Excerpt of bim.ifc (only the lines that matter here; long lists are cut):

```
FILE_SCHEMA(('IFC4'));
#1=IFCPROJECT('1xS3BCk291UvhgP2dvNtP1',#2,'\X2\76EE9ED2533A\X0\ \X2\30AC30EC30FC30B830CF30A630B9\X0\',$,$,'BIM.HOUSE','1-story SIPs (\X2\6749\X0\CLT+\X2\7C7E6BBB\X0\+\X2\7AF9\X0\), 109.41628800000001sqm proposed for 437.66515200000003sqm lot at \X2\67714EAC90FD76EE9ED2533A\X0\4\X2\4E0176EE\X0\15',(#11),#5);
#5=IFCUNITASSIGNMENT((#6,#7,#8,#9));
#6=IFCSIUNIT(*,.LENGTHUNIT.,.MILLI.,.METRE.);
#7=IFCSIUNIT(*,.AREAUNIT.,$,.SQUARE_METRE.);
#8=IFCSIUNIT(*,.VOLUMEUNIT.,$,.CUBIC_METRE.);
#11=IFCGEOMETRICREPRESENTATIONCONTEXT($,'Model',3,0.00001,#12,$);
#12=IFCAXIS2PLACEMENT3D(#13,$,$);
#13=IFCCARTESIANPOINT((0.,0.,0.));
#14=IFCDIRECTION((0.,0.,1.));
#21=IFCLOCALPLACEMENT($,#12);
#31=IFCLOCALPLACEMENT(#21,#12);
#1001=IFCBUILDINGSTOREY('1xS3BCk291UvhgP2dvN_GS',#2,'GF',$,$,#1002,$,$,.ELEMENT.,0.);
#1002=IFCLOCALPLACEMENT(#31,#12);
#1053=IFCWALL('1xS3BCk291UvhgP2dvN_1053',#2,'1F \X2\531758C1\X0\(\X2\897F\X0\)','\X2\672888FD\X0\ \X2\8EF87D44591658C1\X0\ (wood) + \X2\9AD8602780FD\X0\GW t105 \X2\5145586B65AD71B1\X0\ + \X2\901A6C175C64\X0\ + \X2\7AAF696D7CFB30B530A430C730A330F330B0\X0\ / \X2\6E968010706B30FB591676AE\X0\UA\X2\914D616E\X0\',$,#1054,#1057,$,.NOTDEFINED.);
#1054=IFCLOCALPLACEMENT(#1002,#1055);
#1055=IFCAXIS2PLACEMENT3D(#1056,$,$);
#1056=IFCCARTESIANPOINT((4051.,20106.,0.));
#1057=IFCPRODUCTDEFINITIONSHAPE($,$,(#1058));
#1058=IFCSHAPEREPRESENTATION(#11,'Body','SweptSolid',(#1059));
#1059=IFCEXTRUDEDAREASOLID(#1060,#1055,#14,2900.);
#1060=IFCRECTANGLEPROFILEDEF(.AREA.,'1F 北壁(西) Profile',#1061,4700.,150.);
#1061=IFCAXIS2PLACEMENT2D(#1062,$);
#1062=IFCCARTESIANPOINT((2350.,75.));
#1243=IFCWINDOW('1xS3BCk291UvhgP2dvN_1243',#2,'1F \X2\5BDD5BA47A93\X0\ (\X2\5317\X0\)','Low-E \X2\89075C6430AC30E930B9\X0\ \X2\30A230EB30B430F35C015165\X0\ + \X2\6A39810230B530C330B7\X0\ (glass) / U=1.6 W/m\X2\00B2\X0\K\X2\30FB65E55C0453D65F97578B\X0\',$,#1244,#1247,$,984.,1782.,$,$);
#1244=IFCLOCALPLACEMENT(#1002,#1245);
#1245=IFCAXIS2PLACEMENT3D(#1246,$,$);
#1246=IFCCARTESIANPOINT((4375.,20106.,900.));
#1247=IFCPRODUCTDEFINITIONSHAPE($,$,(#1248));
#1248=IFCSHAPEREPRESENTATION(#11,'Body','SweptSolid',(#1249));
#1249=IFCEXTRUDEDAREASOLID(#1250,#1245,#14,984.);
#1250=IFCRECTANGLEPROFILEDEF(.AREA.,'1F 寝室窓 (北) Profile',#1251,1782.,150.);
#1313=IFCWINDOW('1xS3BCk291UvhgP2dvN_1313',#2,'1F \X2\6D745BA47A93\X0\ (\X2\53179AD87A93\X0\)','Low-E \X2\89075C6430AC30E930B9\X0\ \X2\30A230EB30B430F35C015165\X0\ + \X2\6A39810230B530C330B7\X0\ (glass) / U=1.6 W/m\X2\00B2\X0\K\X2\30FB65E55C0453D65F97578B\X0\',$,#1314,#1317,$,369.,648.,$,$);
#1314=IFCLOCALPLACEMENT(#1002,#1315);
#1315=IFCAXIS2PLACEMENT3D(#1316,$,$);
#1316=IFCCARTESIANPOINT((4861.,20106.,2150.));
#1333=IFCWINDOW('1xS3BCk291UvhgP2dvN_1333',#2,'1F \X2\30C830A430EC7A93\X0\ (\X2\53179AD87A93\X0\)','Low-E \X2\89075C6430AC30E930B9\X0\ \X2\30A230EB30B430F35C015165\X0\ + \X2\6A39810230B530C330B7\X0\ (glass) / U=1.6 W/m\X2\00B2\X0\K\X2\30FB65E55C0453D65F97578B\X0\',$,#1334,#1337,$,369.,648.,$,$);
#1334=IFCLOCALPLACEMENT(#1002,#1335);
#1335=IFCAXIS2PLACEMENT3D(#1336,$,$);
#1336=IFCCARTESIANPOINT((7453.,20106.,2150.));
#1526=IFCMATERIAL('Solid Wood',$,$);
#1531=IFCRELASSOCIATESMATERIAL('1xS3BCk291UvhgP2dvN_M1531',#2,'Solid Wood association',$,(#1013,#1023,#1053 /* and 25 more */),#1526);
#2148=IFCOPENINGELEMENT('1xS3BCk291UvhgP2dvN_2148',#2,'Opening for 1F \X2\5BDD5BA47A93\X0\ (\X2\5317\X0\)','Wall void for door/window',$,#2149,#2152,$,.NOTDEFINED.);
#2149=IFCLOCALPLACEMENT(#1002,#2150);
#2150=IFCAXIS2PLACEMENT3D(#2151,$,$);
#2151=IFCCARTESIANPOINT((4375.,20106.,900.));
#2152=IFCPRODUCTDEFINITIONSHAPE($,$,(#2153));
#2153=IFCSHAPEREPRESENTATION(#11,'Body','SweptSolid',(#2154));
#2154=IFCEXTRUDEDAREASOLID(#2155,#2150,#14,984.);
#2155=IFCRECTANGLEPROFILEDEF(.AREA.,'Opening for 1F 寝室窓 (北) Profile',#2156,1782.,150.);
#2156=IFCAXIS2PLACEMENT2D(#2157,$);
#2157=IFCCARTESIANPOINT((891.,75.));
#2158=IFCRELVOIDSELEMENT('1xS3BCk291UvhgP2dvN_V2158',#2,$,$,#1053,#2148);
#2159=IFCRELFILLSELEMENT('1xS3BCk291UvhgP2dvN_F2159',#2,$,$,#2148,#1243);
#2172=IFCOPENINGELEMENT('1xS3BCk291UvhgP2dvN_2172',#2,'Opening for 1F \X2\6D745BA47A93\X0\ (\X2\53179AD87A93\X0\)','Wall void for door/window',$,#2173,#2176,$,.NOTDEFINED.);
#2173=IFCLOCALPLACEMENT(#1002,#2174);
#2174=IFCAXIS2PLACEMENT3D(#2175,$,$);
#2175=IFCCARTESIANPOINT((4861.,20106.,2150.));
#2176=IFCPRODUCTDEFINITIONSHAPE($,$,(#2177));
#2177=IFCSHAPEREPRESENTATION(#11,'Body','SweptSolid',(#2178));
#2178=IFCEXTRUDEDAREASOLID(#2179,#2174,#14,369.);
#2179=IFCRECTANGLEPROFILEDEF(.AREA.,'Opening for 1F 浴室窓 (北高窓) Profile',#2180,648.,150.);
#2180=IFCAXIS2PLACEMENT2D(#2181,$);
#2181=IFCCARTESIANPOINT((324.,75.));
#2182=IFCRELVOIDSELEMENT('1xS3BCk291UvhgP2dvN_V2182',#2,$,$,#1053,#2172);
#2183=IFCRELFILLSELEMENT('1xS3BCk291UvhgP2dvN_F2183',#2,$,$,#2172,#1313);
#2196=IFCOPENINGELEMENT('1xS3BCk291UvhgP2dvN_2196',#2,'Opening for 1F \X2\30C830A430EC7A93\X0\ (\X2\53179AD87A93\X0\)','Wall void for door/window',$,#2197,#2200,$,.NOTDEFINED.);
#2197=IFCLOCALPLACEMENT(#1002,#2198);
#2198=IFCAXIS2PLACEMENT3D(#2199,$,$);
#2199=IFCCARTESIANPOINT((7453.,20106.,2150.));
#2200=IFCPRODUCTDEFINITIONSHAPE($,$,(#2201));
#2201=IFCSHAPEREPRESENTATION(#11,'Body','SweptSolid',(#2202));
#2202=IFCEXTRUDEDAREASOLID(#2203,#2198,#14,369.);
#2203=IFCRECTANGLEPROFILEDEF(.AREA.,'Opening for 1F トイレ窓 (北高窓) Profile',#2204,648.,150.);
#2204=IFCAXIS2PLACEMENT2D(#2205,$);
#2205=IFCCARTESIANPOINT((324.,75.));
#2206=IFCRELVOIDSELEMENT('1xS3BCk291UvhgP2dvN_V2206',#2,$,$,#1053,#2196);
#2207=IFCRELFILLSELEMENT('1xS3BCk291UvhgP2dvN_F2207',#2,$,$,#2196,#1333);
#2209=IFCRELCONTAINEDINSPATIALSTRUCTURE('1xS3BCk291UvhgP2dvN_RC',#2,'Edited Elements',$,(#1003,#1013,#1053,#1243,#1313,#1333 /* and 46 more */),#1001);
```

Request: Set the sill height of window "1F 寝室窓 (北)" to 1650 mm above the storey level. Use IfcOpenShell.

```python
import numpy as np
import ifcopenshell
import ifcopenshell.api.geometry
import ifcopenshell.geom
import ifcopenshell.util.element
import ifcopenshell.util.placement
import ifcopenshell.util.shape
import ifcopenshell.util.unit

model = ifcopenshell.open("bim.ifc")
unit_scale = ifcopenshell.util.unit.calculate_unit_scale(model)

window = model.by_guid("1xS3BCk291UvhgP2dvN_1243")
opening = window.FillsVoids[0].RelatingOpeningElement
storey = ifcopenshell.util.element.get_container(window, ifc_class="IfcBuildingStorey")
level = ifcopenshell.util.placement.get_local_placement(storey.ObjectPlacement)[2, 3]

# The opening's origin need not be at the sill, so measure its lowest point.
shape = ifcopenshell.geom.create_shape(ifcopenshell.geom.settings(), opening)
bottom = ifcopenshell.util.shape.get_shape_bottom_elevation(shape, shape.geometry) / unit_scale
dz = level + 1.65 / unit_scale - bottom

shift = np.array([0.0, 0.0, dz])
# The window is not placed relative to its opening, so move both.
for product in (opening, window):
    matrix = ifcopenshell.util.placement.get_local_placement(product.ObjectPlacement)
    matrix[:3, 3] += shift
    ifcopenshell.api.geometry.edit_object_placement(model, product=product, matrix=matrix, is_si=False)

print(f"moved by {dz * unit_scale:+.3f} m")

model.write("bim_rev.ifc")
```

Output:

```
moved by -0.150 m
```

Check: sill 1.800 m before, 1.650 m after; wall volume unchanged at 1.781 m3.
